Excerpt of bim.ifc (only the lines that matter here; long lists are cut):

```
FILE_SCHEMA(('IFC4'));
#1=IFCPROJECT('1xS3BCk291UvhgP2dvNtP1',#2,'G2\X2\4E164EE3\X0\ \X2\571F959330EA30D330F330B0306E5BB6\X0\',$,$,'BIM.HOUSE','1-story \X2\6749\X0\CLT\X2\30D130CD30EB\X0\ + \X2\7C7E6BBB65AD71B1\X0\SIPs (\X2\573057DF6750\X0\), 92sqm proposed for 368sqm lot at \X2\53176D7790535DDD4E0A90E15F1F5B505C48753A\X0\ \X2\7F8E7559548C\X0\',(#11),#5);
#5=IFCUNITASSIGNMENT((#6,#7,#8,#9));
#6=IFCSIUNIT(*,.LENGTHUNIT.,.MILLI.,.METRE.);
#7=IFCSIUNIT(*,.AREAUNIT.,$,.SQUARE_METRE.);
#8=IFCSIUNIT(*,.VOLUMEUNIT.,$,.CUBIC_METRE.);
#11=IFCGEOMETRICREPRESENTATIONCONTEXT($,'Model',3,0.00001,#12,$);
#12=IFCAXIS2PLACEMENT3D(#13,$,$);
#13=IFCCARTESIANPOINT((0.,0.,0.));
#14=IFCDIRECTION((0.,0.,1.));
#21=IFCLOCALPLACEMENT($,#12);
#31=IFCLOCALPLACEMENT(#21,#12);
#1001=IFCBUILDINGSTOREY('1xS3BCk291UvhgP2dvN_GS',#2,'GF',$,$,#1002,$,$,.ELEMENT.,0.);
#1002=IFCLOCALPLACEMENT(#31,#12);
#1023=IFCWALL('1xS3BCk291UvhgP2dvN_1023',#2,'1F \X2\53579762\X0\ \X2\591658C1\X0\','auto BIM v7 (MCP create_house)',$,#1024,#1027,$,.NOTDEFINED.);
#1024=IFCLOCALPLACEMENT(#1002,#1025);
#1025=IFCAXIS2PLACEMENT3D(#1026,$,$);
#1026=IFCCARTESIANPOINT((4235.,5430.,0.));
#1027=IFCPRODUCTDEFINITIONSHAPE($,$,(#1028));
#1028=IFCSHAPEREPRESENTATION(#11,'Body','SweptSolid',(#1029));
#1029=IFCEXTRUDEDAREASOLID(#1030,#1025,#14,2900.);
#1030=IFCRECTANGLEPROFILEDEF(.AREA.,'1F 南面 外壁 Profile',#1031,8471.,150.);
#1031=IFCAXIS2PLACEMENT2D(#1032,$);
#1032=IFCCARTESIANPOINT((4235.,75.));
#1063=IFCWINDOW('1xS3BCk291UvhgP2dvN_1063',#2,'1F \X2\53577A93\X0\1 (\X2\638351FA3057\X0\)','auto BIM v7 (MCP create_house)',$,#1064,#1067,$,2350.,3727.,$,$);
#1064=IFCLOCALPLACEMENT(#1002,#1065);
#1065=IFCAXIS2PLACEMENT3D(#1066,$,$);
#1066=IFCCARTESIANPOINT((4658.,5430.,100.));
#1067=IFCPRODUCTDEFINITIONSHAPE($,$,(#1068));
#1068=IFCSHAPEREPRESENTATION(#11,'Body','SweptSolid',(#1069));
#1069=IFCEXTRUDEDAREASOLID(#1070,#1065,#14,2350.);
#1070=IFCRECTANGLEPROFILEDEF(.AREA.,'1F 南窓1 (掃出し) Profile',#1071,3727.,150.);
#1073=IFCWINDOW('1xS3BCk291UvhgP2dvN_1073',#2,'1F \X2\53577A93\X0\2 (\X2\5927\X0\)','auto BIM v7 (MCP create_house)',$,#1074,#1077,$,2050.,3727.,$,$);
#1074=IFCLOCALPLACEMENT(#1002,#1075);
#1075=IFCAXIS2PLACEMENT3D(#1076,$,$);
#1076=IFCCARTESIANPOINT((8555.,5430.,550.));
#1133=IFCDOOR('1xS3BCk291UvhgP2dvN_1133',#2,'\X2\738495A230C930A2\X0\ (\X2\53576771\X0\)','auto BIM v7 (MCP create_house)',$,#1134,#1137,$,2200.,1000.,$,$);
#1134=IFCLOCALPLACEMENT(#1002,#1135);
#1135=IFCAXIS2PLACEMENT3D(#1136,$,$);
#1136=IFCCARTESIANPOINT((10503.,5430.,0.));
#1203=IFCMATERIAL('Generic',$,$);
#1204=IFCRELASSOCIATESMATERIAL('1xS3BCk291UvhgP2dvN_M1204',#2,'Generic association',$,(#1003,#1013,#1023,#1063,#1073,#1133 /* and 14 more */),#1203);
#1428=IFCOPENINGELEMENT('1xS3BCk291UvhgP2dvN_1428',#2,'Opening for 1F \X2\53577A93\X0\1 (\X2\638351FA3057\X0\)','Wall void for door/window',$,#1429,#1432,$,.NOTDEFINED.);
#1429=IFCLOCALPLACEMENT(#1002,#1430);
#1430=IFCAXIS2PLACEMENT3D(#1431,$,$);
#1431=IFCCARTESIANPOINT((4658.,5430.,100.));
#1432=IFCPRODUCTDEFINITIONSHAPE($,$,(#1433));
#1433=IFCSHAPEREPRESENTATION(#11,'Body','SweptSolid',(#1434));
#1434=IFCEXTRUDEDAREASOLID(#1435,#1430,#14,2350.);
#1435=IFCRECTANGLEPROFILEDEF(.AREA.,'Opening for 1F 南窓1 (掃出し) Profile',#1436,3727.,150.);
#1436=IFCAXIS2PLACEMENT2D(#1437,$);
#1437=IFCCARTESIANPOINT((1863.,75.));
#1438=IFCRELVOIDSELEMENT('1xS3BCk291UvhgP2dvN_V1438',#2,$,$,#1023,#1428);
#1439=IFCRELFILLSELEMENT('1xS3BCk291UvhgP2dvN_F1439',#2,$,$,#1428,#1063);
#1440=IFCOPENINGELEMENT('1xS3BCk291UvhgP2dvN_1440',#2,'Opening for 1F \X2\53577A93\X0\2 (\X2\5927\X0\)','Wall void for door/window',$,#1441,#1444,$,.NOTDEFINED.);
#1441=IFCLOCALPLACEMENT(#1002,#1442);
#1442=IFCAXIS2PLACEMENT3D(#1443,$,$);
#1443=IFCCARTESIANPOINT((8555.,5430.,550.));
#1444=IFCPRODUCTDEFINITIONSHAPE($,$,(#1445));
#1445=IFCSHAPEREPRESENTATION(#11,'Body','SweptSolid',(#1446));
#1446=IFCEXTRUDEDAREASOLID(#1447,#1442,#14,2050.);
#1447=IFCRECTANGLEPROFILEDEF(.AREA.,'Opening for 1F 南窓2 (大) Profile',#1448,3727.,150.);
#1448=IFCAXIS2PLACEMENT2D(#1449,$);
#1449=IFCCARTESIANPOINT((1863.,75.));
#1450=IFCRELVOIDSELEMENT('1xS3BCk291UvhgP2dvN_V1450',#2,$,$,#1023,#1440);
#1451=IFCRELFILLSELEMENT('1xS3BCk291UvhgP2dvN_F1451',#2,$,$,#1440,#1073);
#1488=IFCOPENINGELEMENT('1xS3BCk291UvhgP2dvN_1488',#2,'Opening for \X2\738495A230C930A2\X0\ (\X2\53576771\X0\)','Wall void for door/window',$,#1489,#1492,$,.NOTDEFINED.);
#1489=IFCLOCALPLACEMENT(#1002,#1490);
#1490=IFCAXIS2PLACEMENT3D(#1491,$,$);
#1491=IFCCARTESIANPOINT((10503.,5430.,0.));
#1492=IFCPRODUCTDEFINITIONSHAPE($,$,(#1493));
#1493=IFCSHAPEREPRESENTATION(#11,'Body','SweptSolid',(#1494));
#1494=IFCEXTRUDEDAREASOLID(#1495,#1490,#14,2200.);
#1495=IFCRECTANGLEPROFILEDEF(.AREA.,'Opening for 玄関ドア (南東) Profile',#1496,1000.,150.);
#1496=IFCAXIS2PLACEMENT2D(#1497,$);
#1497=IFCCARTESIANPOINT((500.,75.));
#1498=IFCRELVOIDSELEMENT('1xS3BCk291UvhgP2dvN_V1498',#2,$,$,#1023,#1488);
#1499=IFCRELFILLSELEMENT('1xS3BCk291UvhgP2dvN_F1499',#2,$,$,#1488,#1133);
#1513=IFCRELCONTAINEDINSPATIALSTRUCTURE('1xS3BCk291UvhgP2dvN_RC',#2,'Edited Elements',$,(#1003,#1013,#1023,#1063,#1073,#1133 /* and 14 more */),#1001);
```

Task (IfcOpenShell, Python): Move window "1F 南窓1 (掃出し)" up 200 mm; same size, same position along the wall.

```python
import numpy as np
import ifcopenshell
import ifcopenshell.api.geometry
import ifcopenshell.util.placement
import ifcopenshell.util.unit

model = ifcopenshell.open("bim.ifc")
unit_scale = ifcopenshell.util.unit.calculate_unit_scale(model)

window = model.by_id(1063)
opening = window.FillsVoids[0].RelatingOpeningElement
dz = 0.2 / unit_scale

shift = np.array([0.0, 0.0, dz])
# The window is not placed relative to its opening, so move both.
for product in (opening, window):
    matrix = ifcopenshell.util.placement.get_local_placement(product.ObjectPlacement)
    matrix[:3, 3] += shift
    ifcopenshell.api.geometry.edit_object_placement(model, product=product, matrix=matrix, is_si=False)

print(f"moved by {dz * unit_scale:+.3f} m")

model.write("bim-out.ifc")
```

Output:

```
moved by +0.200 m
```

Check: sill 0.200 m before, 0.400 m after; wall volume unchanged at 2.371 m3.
